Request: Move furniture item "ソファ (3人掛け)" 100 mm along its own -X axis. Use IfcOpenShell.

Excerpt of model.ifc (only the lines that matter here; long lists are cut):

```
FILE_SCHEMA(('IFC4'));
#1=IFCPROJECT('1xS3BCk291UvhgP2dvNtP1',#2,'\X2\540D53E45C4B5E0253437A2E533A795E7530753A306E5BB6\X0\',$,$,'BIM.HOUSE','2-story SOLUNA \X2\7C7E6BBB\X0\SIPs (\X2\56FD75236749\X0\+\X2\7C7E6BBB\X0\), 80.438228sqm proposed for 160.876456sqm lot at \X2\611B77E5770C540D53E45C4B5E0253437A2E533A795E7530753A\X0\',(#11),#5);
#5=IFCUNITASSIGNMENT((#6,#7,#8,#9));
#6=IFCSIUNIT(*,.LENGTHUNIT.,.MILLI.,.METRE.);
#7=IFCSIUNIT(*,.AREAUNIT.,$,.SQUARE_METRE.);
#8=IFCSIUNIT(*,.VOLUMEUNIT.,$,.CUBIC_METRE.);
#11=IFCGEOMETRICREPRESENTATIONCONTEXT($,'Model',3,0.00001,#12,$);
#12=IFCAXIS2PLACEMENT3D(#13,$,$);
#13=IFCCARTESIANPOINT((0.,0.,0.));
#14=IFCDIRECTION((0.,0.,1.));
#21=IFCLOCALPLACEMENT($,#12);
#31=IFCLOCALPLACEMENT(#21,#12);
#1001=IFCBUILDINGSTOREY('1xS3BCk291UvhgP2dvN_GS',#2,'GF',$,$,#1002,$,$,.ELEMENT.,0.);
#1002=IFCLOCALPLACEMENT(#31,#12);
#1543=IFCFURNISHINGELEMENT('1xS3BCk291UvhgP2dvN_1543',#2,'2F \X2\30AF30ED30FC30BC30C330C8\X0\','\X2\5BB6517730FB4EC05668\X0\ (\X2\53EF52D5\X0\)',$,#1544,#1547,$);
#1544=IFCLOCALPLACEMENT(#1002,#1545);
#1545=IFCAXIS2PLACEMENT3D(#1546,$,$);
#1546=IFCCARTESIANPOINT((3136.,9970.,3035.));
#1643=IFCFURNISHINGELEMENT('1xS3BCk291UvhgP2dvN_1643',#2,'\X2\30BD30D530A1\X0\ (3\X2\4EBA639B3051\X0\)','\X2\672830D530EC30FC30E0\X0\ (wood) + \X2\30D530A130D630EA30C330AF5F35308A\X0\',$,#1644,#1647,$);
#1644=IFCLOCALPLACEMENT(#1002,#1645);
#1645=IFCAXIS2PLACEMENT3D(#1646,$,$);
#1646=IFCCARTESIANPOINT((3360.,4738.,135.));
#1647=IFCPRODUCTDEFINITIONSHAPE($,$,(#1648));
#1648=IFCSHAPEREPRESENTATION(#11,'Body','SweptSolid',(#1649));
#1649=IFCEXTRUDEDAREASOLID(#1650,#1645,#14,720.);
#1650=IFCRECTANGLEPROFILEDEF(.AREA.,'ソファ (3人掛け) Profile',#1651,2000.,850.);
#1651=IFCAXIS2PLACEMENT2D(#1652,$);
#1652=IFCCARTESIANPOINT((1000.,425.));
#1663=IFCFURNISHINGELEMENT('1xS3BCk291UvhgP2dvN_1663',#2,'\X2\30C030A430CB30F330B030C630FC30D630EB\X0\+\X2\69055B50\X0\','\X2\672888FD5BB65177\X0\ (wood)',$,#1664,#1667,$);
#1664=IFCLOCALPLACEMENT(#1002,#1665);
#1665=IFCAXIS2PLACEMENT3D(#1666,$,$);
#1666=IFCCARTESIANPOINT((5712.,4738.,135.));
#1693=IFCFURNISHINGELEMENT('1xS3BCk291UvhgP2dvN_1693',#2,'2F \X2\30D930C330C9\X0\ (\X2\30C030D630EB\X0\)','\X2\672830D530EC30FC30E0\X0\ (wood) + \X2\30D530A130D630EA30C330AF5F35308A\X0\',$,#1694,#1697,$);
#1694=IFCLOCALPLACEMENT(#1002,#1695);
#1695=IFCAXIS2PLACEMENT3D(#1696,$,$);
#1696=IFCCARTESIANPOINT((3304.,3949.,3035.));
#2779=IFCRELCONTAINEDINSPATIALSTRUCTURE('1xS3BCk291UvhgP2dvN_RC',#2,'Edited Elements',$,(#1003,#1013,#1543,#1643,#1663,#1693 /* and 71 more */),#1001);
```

```python
import ifcopenshell
import ifcopenshell.api.geometry
import ifcopenshell.util.placement

model = ifcopenshell.open("model.ifc")

item = model.by_id(1643)
matrix = ifcopenshell.util.placement.get_local_placement(item.ObjectPlacement)
matrix[:3, 3] -= matrix[:3, 0] * 100.0
ifcopenshell.api.geometry.edit_object_placement(model, product=item, matrix=matrix, is_si=False)

print(ifcopenshell.util.placement.get_local_placement(item.ObjectPlacement).round(3) + 0.0)

model.write("model_updated.ifc")
```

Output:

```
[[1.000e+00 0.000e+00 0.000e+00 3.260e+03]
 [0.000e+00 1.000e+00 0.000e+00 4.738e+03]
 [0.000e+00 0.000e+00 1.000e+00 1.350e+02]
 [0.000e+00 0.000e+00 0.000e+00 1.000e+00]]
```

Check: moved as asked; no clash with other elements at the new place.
